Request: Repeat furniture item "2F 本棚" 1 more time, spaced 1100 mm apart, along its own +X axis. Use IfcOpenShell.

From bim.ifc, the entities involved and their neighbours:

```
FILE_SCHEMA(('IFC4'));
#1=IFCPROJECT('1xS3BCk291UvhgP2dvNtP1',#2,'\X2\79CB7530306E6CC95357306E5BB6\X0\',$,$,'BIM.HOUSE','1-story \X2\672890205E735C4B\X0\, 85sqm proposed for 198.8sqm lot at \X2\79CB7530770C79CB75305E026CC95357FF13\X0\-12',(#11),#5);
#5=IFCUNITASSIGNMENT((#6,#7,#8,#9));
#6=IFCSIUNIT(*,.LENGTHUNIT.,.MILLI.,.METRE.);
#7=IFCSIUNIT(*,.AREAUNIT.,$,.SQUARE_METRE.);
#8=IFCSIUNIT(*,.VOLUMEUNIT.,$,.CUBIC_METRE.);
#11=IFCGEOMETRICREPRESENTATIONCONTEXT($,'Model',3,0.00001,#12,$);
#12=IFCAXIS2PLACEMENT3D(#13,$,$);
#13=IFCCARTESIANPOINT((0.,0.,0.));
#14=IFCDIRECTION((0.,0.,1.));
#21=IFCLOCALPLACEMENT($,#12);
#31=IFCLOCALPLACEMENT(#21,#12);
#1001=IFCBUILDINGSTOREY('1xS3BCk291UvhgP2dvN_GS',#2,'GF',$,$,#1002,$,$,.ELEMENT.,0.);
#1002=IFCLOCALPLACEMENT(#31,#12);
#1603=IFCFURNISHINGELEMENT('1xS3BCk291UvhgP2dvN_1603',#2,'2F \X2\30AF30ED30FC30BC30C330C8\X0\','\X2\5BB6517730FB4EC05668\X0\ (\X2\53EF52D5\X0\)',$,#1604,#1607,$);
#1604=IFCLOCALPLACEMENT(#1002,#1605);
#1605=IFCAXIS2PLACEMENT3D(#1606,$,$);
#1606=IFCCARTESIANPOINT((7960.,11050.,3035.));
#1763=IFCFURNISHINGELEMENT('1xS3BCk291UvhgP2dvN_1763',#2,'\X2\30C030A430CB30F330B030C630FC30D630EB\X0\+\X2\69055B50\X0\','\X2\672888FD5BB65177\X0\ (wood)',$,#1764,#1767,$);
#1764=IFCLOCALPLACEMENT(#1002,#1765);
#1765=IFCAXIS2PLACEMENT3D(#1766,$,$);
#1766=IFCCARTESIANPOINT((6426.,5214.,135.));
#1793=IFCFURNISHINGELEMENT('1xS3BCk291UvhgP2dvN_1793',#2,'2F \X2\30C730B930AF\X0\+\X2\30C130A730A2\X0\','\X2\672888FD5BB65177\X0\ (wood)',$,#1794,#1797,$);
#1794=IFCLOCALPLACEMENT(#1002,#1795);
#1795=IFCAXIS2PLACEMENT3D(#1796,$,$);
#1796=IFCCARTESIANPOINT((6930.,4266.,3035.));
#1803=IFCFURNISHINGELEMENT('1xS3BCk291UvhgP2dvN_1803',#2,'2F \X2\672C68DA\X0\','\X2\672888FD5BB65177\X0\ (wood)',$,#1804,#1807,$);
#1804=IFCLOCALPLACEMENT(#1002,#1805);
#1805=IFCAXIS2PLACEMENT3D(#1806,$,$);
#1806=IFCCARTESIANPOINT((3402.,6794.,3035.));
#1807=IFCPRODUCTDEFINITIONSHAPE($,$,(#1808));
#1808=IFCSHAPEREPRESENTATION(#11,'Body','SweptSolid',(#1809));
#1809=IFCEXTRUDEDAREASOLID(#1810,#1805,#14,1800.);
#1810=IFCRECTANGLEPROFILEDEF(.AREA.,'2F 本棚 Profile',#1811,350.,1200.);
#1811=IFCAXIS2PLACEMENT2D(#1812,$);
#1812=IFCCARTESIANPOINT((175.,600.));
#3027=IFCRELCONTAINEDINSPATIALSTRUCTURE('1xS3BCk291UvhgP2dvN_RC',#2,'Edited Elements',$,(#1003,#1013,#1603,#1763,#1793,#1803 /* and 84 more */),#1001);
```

```python
import ifcopenshell
import ifcopenshell.api.geometry
import ifcopenshell.api.root
import ifcopenshell.util.element
import ifcopenshell.util.placement
import ifcopenshell.util.unit

model = ifcopenshell.open("bim.ifc")
unit_scale = ifcopenshell.util.unit.calculate_unit_scale(model)


def reuse_history(source, copy):
    """copy_class also copies each property set's owner history, people and application; keep the originals."""
    for rel in copy.IsDefinedBy:
        if rel.is_a("IfcRelDefinesByProperties") and (history := rel.RelatingPropertyDefinition.OwnerHistory):
            rel.RelatingPropertyDefinition.OwnerHistory = source.OwnerHistory
            ifcopenshell.util.element.remove_deep2(model, history)


source = model.by_guid("1xS3BCk291UvhgP2dvN_1803")
base = ifcopenshell.util.placement.get_local_placement(source.ObjectPlacement)
step = base[:3, 0] * 1.1 / unit_scale

for i in range(1, 2):
    copy = ifcopenshell.api.root.copy_class(model, product=source)
    copy.Representation = ifcopenshell.util.element.copy_deep(
        model, source.Representation, exclude=["IfcGeometricRepresentationContext", "IfcRepresentationMap"]
    )
    reuse_history(source, copy)
    matrix = base.copy()
    matrix[:3, 3] += i * step
    print("added at", matrix[:3, 3].round(3) + 0.0)
    ifcopenshell.api.geometry.edit_object_placement(model, product=copy, matrix=matrix, is_si=False)

model.write("bim_v2.ifc")
```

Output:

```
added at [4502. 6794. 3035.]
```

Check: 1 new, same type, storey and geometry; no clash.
